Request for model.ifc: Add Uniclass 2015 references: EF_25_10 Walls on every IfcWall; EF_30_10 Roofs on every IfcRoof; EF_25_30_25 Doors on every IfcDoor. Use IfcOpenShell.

First a look at what the model holds.

```python
import ifcopenshell

model = ifcopenshell.open("model.ifc")
print(model.schema)
print("classifications:", [c.Name for c in model.by_type("IfcClassification")])
for ifc_class in ("IfcDoor", "IfcRoof", "IfcStair", "IfcWall", "IfcWindow"):
    print(ifc_class, len(model.by_type(ifc_class)))
```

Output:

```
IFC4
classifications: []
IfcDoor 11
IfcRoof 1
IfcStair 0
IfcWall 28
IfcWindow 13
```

```python
import ifcopenshell
import ifcopenshell.api.classification

model = ifcopenshell.open("model.ifc")

system = ifcopenshell.api.classification.add_classification(model, classification="Uniclass 2015")

codes = {
    "IfcWall": ("EF_25_10", "Walls"),
    "IfcRoof": ("EF_30_10", "Roofs"),
    "IfcDoor": ("EF_25_30_25", "Doors"),
}
for ifc_class, (code, name) in codes.items():
    products = model.by_type(ifc_class)
    ifcopenshell.api.classification.add_reference(
        model, products=products, classification=system, identification=code, name=name
    )
    print(code, len(products))

model.write("model_updated.ifc")
```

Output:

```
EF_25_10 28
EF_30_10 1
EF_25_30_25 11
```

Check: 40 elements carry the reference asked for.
